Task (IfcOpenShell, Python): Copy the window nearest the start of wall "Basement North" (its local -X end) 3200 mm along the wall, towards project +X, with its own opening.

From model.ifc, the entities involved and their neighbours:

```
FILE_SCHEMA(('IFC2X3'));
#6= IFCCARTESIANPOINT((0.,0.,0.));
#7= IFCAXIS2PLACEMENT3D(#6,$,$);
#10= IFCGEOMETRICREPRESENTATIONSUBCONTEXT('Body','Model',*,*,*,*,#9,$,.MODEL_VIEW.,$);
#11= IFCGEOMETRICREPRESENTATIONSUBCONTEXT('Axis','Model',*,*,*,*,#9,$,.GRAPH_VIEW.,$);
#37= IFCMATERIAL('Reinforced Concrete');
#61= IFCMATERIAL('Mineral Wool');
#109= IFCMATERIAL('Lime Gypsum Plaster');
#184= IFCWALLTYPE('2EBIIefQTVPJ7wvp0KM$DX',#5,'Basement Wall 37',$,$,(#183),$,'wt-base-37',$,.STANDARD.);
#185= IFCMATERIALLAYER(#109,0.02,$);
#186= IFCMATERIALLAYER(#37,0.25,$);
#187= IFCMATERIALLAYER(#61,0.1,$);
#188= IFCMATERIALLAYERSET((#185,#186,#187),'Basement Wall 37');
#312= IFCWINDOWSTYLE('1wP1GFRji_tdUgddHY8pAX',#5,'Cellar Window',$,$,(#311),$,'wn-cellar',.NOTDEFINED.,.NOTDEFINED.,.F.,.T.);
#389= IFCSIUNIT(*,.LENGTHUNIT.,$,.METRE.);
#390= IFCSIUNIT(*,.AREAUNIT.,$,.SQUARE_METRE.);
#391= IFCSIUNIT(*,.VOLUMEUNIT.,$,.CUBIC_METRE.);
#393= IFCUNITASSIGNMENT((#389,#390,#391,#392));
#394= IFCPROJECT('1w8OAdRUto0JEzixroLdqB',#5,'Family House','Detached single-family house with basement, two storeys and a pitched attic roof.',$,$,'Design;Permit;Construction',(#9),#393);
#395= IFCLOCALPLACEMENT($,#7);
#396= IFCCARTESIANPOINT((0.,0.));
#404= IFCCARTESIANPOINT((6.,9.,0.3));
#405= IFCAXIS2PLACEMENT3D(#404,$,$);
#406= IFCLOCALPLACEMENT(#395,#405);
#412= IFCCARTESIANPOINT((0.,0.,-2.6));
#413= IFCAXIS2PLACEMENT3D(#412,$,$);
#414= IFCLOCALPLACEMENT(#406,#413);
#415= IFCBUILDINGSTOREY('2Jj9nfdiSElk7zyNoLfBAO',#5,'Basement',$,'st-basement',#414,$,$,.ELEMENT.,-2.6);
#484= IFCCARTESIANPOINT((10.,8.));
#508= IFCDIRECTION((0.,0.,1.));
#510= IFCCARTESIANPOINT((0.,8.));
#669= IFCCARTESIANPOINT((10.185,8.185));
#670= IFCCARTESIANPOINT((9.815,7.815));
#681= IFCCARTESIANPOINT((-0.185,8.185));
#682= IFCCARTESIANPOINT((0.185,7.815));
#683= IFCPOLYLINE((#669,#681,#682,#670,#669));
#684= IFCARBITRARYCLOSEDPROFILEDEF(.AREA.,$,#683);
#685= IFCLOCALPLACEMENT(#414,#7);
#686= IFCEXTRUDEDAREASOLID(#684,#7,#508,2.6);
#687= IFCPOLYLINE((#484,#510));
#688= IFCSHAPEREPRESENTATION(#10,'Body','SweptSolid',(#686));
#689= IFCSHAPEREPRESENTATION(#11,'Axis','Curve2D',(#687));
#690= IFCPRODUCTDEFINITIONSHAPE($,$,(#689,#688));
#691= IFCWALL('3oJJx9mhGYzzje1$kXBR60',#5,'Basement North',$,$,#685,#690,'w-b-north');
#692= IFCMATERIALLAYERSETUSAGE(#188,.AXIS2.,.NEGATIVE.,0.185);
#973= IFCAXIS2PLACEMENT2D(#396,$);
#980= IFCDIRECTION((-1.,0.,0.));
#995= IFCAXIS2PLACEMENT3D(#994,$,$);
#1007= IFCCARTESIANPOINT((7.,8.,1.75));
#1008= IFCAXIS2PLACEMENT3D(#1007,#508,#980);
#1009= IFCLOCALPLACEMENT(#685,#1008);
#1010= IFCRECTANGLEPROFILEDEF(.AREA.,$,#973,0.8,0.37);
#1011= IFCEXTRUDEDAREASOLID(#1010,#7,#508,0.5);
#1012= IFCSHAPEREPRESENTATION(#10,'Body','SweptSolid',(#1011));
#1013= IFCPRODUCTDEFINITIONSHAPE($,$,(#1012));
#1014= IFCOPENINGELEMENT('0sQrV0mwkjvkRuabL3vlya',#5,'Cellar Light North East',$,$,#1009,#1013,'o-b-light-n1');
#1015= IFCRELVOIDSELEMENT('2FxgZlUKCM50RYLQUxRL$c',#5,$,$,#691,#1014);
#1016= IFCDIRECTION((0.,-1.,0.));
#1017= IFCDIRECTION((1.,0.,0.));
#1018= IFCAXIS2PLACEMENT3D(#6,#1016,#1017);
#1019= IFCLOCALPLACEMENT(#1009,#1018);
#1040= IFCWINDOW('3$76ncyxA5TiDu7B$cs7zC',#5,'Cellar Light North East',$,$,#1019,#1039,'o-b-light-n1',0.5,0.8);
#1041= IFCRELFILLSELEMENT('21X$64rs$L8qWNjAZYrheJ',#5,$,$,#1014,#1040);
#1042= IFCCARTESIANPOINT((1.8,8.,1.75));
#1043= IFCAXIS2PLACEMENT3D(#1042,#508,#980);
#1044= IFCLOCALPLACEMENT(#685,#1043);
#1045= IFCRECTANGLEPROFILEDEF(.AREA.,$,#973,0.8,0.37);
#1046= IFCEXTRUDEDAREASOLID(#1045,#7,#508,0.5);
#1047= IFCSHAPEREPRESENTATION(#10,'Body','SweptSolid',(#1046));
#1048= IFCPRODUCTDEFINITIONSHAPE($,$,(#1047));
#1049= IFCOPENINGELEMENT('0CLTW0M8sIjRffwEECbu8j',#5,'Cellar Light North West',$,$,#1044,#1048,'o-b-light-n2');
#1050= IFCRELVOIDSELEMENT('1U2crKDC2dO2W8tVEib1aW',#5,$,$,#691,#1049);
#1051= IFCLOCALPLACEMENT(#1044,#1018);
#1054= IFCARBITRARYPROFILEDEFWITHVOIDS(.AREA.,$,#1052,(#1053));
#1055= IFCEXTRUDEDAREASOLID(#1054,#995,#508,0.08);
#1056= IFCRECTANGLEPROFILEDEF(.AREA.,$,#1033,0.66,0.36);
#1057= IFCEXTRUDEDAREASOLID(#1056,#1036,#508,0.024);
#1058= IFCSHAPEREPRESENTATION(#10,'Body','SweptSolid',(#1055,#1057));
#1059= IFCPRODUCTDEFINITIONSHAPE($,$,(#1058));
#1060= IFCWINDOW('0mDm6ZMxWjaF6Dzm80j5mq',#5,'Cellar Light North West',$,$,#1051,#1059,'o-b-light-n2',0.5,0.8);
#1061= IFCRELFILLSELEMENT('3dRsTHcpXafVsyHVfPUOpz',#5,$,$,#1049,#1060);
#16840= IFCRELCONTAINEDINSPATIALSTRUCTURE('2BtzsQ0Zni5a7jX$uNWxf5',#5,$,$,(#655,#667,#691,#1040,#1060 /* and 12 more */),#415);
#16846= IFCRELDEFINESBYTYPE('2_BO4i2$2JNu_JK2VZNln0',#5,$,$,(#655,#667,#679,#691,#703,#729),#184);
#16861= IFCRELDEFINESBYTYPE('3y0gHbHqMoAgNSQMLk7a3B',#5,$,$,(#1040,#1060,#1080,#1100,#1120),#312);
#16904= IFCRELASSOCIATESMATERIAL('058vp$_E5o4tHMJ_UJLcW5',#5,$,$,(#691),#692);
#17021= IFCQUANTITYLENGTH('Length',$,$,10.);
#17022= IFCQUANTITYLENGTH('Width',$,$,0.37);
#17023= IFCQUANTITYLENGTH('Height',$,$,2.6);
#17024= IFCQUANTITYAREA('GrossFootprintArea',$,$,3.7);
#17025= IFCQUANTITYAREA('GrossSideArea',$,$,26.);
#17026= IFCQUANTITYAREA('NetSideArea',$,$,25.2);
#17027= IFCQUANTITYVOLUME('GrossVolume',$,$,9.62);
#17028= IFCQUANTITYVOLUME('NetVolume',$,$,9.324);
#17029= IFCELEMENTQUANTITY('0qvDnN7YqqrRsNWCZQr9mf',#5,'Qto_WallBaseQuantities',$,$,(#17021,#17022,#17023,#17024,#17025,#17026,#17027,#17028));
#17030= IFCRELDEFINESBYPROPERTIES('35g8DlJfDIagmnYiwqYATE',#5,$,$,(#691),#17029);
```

```python
import ifcopenshell
import ifcopenshell.api.feature
import ifcopenshell.api.geometry
import ifcopenshell.api.pset
import ifcopenshell.api.root
import ifcopenshell.geom
import ifcopenshell.util.element
import ifcopenshell.util.placement
import ifcopenshell.util.shape
import ifcopenshell.util.unit

model = ifcopenshell.open("model.ifc")
unit_scale = ifcopenshell.util.unit.calculate_unit_scale(model)
area_scale = ifcopenshell.util.unit.calculate_unit_scale(model, "AREAUNIT")
volume_scale = ifcopenshell.util.unit.calculate_unit_scale(model, "VOLUMEUNIT")
settings = ifcopenshell.geom.settings()


def volume(element):
    """Net volume in cubic metres, openings subtracted."""
    shape = ifcopenshell.geom.create_shape(settings, element)
    return ifcopenshell.util.shape.get_volume(shape.geometry)


def reuse_history(source, copy):
    """copy_class also copies each property set's owner history, people and application; keep the originals."""
    for rel in copy.IsDefinedBy:
        if rel.is_a("IfcRelDefinesByProperties") and (history := rel.RelatingPropertyDefinition.OwnerHistory):
            rel.RelatingPropertyDefinition.OwnerHistory = source.OwnerHistory
            ifcopenshell.util.element.remove_deep2(model, history)


window = model.by_guid("0mDm6ZMxWjaF6Dzm80j5mq")
opening = window.FillsVoids[0].RelatingOpeningElement
wall = opening.VoidsElements[0].RelatingBuildingElement
before = volume(wall)
shift = ifcopenshell.util.placement.get_local_placement(wall.ObjectPlacement)[:3, 0] * 3.2 / unit_scale

# copy_class copies the void relationship, type, container and properties, but no geometry.
new_opening = ifcopenshell.api.root.copy_class(model, product=opening)
new_opening.Representation = ifcopenshell.util.element.copy_deep(
    model, opening.Representation, exclude=["IfcGeometricRepresentationContext", "IfcRepresentationMap"]
)
new_opening.Tag = None
new_window = ifcopenshell.api.root.copy_class(model, product=window)
new_window.Representation = ifcopenshell.util.element.copy_deep(
    model, window.Representation, exclude=["IfcGeometricRepresentationContext", "IfcRepresentationMap"]
)
new_window.Tag = None
reuse_history(window, new_window)
fills = ifcopenshell.api.feature.add_filling(model, opening=new_opening, element=new_window)
fills.OwnerHistory = new_window.OwnerHistory  # required in IFC2X3

for old, new in ((opening, new_opening), (window, new_window)):
    matrix = ifcopenshell.util.placement.get_local_placement(old.ObjectPlacement)
    matrix[:3, 3] += shift
    ifcopenshell.api.geometry.edit_object_placement(model, product=new, matrix=matrix, is_si=False)

after = volume(wall)
thickness = 0.37  # wall thickness in metres

# Update the wall's stored quantities.
qto = model.by_id(ifcopenshell.util.element.get_pset(wall, "Qto_WallBaseQuantities", should_inherit=False)["id"])
ifcopenshell.api.pset.edit_qto(model, qto=qto, properties={
    "NetSideArea": after / thickness / area_scale,
    "NetVolume": after / volume_scale,
})

print(f"wall volume {before:.3f} -> {after:.3f} m3")

model.write("model_edited.ifc")
```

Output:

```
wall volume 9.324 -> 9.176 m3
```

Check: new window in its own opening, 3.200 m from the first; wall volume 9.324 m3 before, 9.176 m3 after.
